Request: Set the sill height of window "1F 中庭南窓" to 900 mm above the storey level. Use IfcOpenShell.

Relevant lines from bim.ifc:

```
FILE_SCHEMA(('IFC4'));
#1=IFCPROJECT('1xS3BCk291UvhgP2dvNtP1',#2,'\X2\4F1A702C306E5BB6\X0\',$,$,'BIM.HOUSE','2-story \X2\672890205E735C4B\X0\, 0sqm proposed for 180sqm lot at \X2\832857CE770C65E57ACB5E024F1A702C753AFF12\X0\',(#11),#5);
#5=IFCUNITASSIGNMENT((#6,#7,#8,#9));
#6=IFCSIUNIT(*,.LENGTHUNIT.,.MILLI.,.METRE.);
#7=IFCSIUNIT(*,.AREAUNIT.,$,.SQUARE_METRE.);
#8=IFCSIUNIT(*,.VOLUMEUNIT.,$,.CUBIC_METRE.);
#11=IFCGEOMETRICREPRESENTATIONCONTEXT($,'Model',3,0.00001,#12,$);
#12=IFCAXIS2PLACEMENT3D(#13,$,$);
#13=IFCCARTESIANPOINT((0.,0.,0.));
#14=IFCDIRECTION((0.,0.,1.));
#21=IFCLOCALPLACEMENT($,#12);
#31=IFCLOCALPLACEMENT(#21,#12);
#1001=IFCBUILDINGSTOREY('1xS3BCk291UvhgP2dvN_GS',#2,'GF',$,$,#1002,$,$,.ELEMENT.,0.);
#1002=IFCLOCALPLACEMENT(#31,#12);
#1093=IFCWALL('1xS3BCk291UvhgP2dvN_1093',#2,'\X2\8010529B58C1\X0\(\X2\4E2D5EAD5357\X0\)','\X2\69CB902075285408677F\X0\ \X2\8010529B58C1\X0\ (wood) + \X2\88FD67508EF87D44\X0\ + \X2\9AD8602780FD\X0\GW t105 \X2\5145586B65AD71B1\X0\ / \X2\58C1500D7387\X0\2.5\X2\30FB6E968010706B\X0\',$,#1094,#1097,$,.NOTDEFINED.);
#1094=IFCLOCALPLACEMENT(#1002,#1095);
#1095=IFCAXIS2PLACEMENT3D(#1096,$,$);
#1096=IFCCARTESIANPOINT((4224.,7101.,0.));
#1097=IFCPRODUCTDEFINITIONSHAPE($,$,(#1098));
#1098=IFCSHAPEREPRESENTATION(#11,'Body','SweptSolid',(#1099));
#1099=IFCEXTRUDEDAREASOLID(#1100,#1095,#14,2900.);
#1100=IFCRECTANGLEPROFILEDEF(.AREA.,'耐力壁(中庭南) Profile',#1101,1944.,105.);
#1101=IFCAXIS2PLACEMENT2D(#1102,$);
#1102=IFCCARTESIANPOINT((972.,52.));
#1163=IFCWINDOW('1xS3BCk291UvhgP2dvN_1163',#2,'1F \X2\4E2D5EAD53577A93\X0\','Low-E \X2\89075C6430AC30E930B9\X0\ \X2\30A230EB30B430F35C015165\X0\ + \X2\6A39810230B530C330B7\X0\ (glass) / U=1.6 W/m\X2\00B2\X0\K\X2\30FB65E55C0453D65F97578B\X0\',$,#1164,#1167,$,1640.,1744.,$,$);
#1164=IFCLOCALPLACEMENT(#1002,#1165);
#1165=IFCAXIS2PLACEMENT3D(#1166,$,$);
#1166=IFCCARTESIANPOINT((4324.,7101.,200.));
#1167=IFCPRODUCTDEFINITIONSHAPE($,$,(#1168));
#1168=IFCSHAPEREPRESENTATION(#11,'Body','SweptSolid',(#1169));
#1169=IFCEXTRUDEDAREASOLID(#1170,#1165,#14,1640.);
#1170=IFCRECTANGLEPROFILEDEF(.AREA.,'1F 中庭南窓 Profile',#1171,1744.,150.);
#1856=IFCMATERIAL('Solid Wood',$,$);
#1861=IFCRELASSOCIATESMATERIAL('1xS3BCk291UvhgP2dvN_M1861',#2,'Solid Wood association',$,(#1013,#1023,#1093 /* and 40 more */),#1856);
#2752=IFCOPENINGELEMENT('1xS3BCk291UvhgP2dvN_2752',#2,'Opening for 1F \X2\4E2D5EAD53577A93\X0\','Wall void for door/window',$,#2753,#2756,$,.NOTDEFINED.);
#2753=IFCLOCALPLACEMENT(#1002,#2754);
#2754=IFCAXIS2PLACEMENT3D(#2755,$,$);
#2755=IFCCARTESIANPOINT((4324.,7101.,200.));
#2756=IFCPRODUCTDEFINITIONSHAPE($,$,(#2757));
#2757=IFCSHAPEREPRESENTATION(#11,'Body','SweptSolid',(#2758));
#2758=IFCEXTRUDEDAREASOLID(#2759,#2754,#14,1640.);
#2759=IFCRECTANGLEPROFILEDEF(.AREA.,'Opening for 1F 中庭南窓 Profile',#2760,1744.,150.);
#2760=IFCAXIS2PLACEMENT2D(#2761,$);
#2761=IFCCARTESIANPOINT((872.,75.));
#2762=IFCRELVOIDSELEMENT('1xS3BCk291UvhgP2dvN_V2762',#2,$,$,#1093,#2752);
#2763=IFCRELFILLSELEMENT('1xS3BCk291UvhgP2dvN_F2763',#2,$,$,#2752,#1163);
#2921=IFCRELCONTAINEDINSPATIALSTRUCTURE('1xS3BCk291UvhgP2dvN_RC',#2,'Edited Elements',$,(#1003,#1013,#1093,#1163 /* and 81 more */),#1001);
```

```python
import numpy as np
import ifcopenshell
import ifcopenshell.api.geometry
import ifcopenshell.geom
import ifcopenshell.util.element
import ifcopenshell.util.placement
import ifcopenshell.util.shape
import ifcopenshell.util.unit

model = ifcopenshell.open("bim.ifc")
unit_scale = ifcopenshell.util.unit.calculate_unit_scale(model)

window = model.by_id(1163)
opening = window.FillsVoids[0].RelatingOpeningElement
storey = ifcopenshell.util.element.get_container(window, ifc_class="IfcBuildingStorey")
level = ifcopenshell.util.placement.get_local_placement(storey.ObjectPlacement)[2, 3]

# The opening's origin need not be at the sill, so measure its lowest point.
shape = ifcopenshell.geom.create_shape(ifcopenshell.geom.settings(), opening)
bottom = ifcopenshell.util.shape.get_shape_bottom_elevation(shape, shape.geometry) / unit_scale
dz = level + 0.9 / unit_scale - bottom

shift = np.array([0.0, 0.0, dz])
# The window is not placed relative to its opening, so move both.
for product in (opening, window):
    matrix = ifcopenshell.util.placement.get_local_placement(product.ObjectPlacement)
    matrix[:3, 3] += shift
    ifcopenshell.api.geometry.edit_object_placement(model, product=product, matrix=matrix, is_si=False)

print(f"moved by {dz * unit_scale:+.3f} m")

model.write("bim_rev.ifc")
```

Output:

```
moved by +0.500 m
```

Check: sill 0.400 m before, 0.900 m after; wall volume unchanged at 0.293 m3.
